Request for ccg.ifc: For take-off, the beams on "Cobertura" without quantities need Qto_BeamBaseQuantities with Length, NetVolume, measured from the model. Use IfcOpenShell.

First a look at what the model holds.

```python
import ifcopenshell
import ifcopenshell.util.element
import ifcopenshell.util.unit

model = ifcopenshell.open("ccg.ifc")
print(model.schema)
for unit_type in ("LENGTHUNIT", "AREAUNIT", "VOLUMEUNIT"):
    print(unit_type, ifcopenshell.util.unit.calculate_unit_scale(model, unit_type))
storey = next(s for s in model.by_type("IfcBuildingStorey") if s.Name == "Cobertura")
beams = [e for e in ifcopenshell.util.element.get_decomposition(storey) if e.is_a("IfcBeam")]
for e in sorted(beams, key=lambda e: e.id()):
    print(e.id(), e.is_a(), e.Name, list(ifcopenshell.util.element.get_psets(e, qtos_only=True)), sep=" | ")
```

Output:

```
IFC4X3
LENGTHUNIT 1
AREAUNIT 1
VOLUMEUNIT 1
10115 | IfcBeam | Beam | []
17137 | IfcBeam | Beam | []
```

```python
import ifcopenshell
import ifcopenshell.api.pset
import ifcopenshell.geom
import ifcopenshell.util.element
import ifcopenshell.util.shape
import ifcopenshell.util.unit

model = ifcopenshell.open("ccg.ifc")
unit_scale = ifcopenshell.util.unit.calculate_unit_scale(model)
volume_scale = ifcopenshell.util.unit.calculate_unit_scale(model, "VOLUMEUNIT")
settings = ifcopenshell.geom.settings()

storey = next(s for s in model.by_type("IfcBuildingStorey") if s.Name == "Cobertura")
beams = [e for e in ifcopenshell.util.element.get_decomposition(storey) if e.is_a("IfcBeam")]

for e in sorted(beams, key=lambda e: e.id()):
    if ifcopenshell.util.element.get_psets(e, qtos_only=True, should_inherit=False):
        continue
    # Geometry comes back in metres, in the element's own axes.
    shape = ifcopenshell.geom.create_shape(settings, e)
    values = {
        "Length": ifcopenshell.util.shape.get_max_xyz(shape.geometry) / unit_scale,
        "NetVolume": ifcopenshell.util.shape.get_volume(shape.geometry) / volume_scale,
    }
    qto = ifcopenshell.api.pset.add_qto(model, product=e, name="Qto_BeamBaseQuantities")
    ifcopenshell.api.pset.edit_qto(model, qto=qto, properties=values)
    print(e.id(), {k: round(v, 3) for k, v in values.items()})

model.write("ccg_rev.ifc")
```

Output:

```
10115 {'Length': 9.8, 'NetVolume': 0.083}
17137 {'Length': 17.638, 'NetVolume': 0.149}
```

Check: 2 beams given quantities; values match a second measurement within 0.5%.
